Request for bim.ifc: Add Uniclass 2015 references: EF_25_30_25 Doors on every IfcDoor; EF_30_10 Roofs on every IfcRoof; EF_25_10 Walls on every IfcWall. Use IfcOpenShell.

First a look at what the model holds.

```python
import ifcopenshell

model = ifcopenshell.open("bim.ifc")
print(model.schema)
print("classifications:", [c.Name for c in model.by_type("IfcClassification")])
for ifc_class in ("IfcDoor", "IfcRoof", "IfcStair", "IfcWall", "IfcWindow"):
    print(ifc_class, len(model.by_type(ifc_class)))
```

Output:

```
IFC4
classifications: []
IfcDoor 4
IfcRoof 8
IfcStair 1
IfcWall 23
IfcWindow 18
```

```python
import ifcopenshell
import ifcopenshell.api.classification

model = ifcopenshell.open("bim.ifc")

system = ifcopenshell.api.classification.add_classification(model, classification="Uniclass 2015")

codes = {
    "IfcDoor": ("EF_25_30_25", "Doors"),
    "IfcRoof": ("EF_30_10", "Roofs"),
    "IfcWall": ("EF_25_10", "Walls"),
}
for ifc_class, (code, name) in codes.items():
    products = model.by_type(ifc_class)
    ifcopenshell.api.classification.add_reference(
        model, products=products, classification=system, identification=code, name=name
    )
    print(code, len(products))

model.write("bim_v2.ifc")
```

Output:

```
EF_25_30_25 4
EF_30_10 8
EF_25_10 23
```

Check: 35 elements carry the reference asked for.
